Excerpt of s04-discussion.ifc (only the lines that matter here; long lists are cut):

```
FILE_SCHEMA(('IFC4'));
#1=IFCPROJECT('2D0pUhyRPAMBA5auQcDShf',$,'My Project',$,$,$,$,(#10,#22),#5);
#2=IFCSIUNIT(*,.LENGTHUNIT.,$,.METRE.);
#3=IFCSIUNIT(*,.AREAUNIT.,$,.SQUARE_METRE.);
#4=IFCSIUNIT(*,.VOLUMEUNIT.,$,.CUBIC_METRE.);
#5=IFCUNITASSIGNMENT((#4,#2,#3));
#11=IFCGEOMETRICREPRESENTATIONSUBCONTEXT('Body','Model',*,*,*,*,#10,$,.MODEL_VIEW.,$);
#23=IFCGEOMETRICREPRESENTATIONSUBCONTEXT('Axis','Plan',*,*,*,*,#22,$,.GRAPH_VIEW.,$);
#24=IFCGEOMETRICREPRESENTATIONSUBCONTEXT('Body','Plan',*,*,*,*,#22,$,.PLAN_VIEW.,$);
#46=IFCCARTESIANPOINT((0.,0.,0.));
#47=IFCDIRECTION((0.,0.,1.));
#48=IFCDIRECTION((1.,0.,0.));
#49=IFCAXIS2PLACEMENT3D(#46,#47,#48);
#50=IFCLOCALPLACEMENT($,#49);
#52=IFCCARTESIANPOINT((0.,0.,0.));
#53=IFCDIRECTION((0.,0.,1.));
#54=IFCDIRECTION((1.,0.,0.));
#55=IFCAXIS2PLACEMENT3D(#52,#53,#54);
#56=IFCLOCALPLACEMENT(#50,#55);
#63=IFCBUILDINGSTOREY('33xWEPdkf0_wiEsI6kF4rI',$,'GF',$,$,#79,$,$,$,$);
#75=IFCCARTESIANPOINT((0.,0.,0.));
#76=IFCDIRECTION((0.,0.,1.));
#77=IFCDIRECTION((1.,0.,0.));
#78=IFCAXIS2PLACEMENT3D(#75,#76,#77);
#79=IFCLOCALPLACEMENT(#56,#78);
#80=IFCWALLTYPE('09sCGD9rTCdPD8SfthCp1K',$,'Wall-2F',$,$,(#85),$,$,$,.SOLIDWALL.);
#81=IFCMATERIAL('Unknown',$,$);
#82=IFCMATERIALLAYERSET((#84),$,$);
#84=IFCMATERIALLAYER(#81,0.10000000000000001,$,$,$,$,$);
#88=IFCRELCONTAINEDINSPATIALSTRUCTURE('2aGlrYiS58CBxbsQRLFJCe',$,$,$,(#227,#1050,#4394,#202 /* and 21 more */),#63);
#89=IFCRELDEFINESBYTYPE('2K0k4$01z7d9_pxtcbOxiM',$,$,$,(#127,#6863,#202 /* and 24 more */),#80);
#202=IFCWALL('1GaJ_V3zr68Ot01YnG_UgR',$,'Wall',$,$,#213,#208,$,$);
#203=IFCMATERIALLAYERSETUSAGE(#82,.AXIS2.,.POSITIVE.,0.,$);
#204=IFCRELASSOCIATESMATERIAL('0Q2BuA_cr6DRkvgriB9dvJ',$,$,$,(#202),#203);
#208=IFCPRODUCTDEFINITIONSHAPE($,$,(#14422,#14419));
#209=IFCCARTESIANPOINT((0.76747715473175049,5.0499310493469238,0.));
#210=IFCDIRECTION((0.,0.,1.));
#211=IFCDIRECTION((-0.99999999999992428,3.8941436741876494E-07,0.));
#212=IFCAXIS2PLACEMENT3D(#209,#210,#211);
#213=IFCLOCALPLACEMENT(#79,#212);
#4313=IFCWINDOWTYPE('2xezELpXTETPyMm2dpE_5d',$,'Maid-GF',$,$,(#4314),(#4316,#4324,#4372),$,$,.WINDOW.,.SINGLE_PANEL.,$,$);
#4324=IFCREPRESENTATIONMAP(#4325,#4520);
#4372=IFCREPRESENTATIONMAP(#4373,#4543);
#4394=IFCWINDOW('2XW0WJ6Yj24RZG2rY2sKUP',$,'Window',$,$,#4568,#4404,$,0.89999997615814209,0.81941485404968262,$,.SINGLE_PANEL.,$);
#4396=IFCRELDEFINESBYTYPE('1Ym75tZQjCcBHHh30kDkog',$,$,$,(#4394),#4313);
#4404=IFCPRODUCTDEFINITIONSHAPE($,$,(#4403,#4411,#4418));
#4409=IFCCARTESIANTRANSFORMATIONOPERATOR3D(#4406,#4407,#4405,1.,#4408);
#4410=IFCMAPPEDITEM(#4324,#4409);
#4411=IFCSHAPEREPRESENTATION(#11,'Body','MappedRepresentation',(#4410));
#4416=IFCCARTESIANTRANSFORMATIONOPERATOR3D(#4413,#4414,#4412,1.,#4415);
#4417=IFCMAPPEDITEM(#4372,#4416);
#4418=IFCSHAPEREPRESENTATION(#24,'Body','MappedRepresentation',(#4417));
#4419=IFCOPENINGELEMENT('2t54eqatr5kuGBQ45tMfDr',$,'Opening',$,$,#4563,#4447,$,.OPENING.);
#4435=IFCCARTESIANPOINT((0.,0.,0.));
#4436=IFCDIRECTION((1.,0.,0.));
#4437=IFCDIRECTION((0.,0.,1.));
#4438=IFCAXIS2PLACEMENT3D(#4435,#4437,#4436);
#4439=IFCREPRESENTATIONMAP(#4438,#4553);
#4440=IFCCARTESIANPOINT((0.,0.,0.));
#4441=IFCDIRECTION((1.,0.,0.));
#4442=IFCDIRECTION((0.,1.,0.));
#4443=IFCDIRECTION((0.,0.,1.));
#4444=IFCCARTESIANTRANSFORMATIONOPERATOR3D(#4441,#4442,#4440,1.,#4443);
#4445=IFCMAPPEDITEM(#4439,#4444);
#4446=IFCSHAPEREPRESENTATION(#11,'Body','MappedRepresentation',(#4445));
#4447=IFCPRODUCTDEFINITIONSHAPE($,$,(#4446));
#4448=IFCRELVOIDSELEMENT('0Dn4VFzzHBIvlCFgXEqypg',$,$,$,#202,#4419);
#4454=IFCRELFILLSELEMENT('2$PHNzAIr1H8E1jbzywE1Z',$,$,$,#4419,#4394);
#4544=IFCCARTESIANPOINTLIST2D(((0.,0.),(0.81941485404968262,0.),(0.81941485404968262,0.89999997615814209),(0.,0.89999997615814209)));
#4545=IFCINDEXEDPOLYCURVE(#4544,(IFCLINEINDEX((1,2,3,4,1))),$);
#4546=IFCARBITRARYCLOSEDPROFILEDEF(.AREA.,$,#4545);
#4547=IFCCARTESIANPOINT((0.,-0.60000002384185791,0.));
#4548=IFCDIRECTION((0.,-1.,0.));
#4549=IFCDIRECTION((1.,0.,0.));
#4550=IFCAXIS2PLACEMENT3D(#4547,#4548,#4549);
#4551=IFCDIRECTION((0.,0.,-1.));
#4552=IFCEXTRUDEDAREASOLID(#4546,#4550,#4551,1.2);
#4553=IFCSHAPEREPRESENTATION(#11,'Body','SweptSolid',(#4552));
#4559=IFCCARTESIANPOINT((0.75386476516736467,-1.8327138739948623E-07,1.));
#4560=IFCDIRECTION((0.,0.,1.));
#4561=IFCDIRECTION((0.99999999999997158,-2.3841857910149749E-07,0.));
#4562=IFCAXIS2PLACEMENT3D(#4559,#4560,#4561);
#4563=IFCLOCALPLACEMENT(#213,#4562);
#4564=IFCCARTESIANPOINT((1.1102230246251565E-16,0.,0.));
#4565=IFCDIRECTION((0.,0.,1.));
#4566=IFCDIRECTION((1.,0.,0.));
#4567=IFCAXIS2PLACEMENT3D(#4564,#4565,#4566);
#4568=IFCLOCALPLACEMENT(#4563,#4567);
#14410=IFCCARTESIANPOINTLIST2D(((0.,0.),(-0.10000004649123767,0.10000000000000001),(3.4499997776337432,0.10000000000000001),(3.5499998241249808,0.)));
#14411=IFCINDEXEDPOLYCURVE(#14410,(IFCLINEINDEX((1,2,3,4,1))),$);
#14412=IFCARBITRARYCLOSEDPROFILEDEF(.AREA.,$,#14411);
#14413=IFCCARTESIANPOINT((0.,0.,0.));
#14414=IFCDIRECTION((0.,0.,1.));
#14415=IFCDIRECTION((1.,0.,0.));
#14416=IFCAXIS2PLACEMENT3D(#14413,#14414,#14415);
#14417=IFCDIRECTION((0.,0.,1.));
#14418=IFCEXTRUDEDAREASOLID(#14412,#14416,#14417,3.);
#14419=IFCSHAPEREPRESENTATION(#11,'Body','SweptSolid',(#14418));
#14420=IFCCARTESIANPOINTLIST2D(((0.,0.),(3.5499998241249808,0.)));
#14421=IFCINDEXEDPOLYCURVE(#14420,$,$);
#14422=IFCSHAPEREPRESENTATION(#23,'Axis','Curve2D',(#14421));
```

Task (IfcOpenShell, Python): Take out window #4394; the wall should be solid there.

```python
import ifcopenshell
import ifcopenshell.api.feature
import ifcopenshell.api.root
import ifcopenshell.geom
import ifcopenshell.util.shape

model = ifcopenshell.open("s04-discussion.ifc")
settings = ifcopenshell.geom.settings()


def volume(element):
    """Net volume in cubic metres, openings subtracted."""
    shape = ifcopenshell.geom.create_shape(settings, element)
    return ifcopenshell.util.shape.get_volume(shape.geometry)


window = model.by_id(4394)
opening = window.FillsVoids[0].RelatingOpeningElement
wall = opening.VoidsElements[0].RelatingBuildingElement
before = volume(wall)

ifcopenshell.api.root.remove_product(model, product=window)
ifcopenshell.api.feature.remove_feature(model, feature=opening)

after = volume(wall)

print(f"wall volume {before:.3f} -> {after:.3f} m3")

model.write("s04-discussion_edited.ifc")
```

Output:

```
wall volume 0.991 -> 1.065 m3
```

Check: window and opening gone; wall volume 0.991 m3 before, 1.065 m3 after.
